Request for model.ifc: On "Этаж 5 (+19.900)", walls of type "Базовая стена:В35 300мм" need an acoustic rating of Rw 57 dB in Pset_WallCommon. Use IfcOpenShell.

First a look at what the model holds.

```python
import ifcopenshell
import ifcopenshell.util.element

model = ifcopenshell.open("model.ifc")
print(model.schema)
storey = next(s for s in model.by_type("IfcBuildingStorey") if s.Name == "Этаж 5 (+19.900)")
walls = [e for e in ifcopenshell.util.element.get_decomposition(storey) if e.is_a("IfcWall")]
seen = {}
for e in walls:
    element_type = ifcopenshell.util.element.get_type(e)
    key = (element_type.Name if element_type != e and element_type else None, ifcopenshell.util.element.get_pset(e, "Pset_WallCommon", "AcousticRating"))
    seen[key] = seen.get(key, 0) + 1
for (name, value), count in sorted(seen.items(), key=str):
    print(count, "x", name, "|", value)
```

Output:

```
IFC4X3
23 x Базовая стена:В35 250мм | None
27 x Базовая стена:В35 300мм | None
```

```python
import ifcopenshell
import ifcopenshell.api.pset
import ifcopenshell.util.element

model = ifcopenshell.open("model.ifc")

storey = next(s for s in model.by_type("IfcBuildingStorey") if s.Name == "Этаж 5 (+19.900)")
walls = [e for e in ifcopenshell.util.element.get_decomposition(storey) if e.is_a("IfcWall")]

count = 0
for e in walls:
    element_type = ifcopenshell.util.element.get_type(e)
    if element_type in (None, e) or element_type.Name != "Базовая стена:В35 300мм":
        continue
    # add_pset returns the element's existing set when there is one.
    pset = ifcopenshell.api.pset.add_pset(model, product=e, name="Pset_WallCommon")
    ifcopenshell.api.pset.edit_pset(model, pset=pset, properties={"AcousticRating": "Rw 57 dB"})
    count += 1

print(count, "walls updated")

model.write("model-out.ifc")
```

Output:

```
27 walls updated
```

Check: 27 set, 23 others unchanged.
